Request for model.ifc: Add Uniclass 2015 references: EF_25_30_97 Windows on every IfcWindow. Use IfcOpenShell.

First a look at what the model holds.

```python
import ifcopenshell

model = ifcopenshell.open("model.ifc")
print(model.schema)
print("classifications:", [c.Name for c in model.by_type("IfcClassification")])
for ifc_class in ("IfcDoor", "IfcRoof", "IfcStair", "IfcWall", "IfcWindow"):
    print(ifc_class, len(model.by_type(ifc_class)))
```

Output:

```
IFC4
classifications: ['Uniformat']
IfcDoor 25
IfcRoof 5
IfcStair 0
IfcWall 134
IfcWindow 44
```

```python
import ifcopenshell
import ifcopenshell.api.classification

model = ifcopenshell.open("model.ifc")

system = ifcopenshell.api.classification.add_classification(model, classification="Uniclass 2015")

codes = {
    "IfcWindow": ("EF_25_30_97", "Windows"),
}
for ifc_class, (code, name) in codes.items():
    products = model.by_type(ifc_class)
    ifcopenshell.api.classification.add_reference(
        model, products=products, classification=system, identification=code, name=name
    )
    print(code, len(products))

model.write("model_rev.ifc")
```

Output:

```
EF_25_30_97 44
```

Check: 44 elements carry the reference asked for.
